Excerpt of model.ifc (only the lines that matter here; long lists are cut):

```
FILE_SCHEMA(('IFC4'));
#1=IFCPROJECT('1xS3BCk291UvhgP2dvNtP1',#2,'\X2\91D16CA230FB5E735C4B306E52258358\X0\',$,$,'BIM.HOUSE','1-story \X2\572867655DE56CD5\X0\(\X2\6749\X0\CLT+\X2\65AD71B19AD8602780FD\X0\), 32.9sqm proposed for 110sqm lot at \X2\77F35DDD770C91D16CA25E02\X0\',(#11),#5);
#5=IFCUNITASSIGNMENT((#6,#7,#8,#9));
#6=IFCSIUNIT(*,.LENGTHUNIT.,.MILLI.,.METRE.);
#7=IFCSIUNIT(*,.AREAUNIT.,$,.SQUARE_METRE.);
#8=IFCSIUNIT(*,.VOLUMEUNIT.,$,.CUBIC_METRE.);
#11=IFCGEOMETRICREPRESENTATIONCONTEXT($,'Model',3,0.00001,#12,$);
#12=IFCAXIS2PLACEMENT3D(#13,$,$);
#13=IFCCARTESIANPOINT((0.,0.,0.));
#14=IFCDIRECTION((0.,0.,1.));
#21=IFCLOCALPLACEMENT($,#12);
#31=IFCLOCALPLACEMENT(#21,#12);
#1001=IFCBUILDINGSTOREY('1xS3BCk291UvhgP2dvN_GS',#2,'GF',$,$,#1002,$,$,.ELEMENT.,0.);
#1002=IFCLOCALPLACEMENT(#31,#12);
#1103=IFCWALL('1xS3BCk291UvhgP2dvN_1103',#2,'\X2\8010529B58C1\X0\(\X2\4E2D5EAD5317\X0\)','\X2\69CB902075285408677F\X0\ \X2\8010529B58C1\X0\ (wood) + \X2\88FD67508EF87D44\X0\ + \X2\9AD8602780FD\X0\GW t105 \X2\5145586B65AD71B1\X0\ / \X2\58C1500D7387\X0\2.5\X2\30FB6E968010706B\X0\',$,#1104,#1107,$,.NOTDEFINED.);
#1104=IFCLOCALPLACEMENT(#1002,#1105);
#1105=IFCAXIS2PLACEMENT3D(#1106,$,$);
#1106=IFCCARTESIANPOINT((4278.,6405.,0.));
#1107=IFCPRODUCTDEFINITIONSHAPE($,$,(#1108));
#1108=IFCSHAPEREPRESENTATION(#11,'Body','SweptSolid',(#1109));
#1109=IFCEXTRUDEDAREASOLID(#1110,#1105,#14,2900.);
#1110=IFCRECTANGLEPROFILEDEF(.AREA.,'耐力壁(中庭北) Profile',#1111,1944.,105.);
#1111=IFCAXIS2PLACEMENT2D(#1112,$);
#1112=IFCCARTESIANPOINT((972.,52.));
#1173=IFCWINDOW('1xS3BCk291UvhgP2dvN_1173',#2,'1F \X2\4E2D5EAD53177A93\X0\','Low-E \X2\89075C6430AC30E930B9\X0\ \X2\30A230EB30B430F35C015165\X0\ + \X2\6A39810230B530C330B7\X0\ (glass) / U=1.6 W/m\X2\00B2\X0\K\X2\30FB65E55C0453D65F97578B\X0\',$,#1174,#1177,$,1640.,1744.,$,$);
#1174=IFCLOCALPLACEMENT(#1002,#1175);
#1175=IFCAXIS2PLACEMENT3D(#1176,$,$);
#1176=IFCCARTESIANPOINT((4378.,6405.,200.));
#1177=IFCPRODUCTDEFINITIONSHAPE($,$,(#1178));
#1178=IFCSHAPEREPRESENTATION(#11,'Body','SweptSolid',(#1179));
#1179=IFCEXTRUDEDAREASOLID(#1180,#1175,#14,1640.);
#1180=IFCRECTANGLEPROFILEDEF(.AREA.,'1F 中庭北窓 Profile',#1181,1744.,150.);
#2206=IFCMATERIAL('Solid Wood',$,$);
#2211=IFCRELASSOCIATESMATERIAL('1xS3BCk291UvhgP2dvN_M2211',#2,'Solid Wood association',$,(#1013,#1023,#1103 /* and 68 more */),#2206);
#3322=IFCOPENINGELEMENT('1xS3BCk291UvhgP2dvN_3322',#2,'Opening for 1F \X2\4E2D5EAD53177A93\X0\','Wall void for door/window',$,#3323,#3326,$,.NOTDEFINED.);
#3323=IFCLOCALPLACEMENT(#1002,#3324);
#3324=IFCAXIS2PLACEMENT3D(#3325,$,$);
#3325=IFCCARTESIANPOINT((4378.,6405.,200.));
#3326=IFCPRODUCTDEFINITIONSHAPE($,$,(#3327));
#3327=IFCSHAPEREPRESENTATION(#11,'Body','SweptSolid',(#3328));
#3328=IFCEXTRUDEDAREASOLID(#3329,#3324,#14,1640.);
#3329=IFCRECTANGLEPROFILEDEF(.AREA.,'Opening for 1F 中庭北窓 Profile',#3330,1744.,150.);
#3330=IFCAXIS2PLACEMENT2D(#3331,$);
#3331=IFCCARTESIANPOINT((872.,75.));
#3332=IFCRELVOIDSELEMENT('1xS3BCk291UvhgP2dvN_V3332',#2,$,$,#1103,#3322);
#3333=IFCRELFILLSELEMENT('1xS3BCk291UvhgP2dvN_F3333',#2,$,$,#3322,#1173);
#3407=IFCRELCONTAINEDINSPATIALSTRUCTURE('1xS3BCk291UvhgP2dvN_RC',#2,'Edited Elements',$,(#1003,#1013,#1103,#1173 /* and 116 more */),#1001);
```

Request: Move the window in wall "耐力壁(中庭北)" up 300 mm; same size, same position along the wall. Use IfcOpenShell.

```python
import numpy as np
import ifcopenshell
import ifcopenshell.api.geometry
import ifcopenshell.util.placement
import ifcopenshell.util.unit

model = ifcopenshell.open("model.ifc")
unit_scale = ifcopenshell.util.unit.calculate_unit_scale(model)

window = model.by_guid("1xS3BCk291UvhgP2dvN_1173")
opening = window.FillsVoids[0].RelatingOpeningElement
dz = 300.0

shift = np.array([0.0, 0.0, dz])
# The window is not placed relative to its opening, so move both.
for product in (opening, window):
    matrix = ifcopenshell.util.placement.get_local_placement(product.ObjectPlacement)
    matrix[:3, 3] += shift
    ifcopenshell.api.geometry.edit_object_placement(model, product=product, matrix=matrix, is_si=False)

print(f"moved by {dz * unit_scale:+.3f} m")

model.write("model-out.ifc")
```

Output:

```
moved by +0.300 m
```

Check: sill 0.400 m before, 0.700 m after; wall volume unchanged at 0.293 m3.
